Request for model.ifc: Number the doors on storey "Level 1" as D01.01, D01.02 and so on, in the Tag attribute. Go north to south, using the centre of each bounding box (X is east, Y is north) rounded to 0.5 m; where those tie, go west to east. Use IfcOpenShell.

First a look at what the model holds.

```python
import ifcopenshell
import ifcopenshell.util.element
import ifcopenshell.util.placement

model = ifcopenshell.open("model.ifc")
print(model.schema)
storey = next(s for s in model.by_type("IfcBuildingStorey") if s.Name == "Level 1")
doors = [e for e in ifcopenshell.util.element.get_decomposition(storey) if e.is_a("IfcDoor")]
for e in sorted(doors, key=lambda e: e.id()):
    origin = ifcopenshell.util.placement.get_local_placement(e.ObjectPlacement)[:3, 3]
    print(e.id(), e.Tag, e.Name, origin.round(2) + 0.0, sep=" | ")
```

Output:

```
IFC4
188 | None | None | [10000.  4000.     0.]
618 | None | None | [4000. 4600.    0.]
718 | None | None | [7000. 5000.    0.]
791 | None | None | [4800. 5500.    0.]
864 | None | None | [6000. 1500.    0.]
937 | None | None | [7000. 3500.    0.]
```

```python
import ifcopenshell
import ifcopenshell.geom
import ifcopenshell.util.element
import ifcopenshell.util.shape

model = ifcopenshell.open("model.ifc")
settings = ifcopenshell.geom.settings()
settings.set("use-world-coords", True)


def centre(element):
    shape = ifcopenshell.geom.create_shape(settings, element)
    return ifcopenshell.util.shape.get_bbox_centroid(shape.geometry)


storey = next(s for s in model.by_type("IfcBuildingStorey") if s.Name == "Level 1")
doors = [e for e in ifcopenshell.util.element.get_decomposition(storey) if e.is_a("IfcDoor")]

# Insertion points can sit at a corner or the storey origin, so sort by the geometry (in metres).
centres = {e: centre(e) for e in doors}
doors.sort(key=lambda e: (-round(centres[e][1] / 0.5), centres[e][0]))

for i, e in enumerate(doors, start=1):
    number = f"D01.{i:02d}"
    e.Tag = number
    print(e.id(), number)

model.write("model-out.ifc")
```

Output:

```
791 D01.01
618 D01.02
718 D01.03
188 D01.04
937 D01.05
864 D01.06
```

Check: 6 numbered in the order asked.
